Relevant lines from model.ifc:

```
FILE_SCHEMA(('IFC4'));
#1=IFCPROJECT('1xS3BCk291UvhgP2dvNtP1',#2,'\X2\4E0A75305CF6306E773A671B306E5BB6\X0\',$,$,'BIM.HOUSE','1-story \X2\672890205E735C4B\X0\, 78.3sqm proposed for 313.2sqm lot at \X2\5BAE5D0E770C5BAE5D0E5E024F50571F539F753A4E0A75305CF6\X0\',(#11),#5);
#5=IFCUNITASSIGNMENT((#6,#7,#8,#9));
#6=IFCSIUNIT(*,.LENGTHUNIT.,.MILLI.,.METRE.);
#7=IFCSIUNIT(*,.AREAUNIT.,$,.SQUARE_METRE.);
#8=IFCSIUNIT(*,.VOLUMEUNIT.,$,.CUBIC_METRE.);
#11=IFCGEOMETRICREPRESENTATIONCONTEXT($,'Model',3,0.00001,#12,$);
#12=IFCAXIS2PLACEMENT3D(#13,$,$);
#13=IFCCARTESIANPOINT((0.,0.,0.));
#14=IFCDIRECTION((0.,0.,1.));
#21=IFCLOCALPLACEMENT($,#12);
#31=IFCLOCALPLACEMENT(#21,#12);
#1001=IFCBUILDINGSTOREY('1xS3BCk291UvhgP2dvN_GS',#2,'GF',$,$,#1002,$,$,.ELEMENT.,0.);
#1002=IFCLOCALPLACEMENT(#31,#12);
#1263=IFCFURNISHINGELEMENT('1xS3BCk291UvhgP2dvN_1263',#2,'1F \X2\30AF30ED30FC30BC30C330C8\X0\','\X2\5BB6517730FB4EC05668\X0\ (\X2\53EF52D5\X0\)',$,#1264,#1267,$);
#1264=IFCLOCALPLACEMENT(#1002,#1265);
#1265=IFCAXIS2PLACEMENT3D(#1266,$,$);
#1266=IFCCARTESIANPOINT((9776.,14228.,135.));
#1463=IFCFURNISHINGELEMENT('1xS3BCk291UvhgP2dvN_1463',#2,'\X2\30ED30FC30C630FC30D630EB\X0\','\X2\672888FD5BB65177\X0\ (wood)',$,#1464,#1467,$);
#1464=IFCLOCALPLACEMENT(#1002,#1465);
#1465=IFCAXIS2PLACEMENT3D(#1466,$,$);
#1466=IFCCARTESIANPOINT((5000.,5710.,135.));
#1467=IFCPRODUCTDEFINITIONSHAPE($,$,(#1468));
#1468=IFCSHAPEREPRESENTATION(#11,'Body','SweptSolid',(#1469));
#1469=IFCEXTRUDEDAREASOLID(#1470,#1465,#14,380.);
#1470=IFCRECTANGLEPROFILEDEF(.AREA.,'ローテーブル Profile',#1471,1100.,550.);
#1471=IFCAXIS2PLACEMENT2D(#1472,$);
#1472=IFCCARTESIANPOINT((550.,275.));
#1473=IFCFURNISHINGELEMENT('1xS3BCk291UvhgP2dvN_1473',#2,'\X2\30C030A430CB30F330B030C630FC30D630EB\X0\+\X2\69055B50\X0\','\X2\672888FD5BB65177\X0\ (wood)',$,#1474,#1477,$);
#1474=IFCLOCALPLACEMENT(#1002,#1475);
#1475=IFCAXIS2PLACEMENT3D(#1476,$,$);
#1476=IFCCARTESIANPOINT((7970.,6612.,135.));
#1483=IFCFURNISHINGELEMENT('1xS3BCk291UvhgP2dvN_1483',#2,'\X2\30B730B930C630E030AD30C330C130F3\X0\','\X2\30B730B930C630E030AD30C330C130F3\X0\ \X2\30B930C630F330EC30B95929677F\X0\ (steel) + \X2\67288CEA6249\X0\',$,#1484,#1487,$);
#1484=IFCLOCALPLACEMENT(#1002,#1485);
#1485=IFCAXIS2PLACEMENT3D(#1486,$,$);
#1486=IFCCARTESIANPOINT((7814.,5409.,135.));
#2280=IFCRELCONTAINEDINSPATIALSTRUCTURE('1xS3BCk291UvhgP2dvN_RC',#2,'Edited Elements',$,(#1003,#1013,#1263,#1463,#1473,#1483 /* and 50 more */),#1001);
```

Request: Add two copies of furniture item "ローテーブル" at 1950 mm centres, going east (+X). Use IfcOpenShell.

```python
import numpy as np
import ifcopenshell
import ifcopenshell.api.geometry
import ifcopenshell.api.root
import ifcopenshell.util.element
import ifcopenshell.util.placement
import ifcopenshell.util.unit

model = ifcopenshell.open("model.ifc")
unit_scale = ifcopenshell.util.unit.calculate_unit_scale(model)


def reuse_history(source, copy):
    """copy_class also copies each property set's owner history, people and application; keep the originals."""
    for rel in copy.IsDefinedBy:
        if rel.is_a("IfcRelDefinesByProperties") and (history := rel.RelatingPropertyDefinition.OwnerHistory):
            rel.RelatingPropertyDefinition.OwnerHistory = source.OwnerHistory
            ifcopenshell.util.element.remove_deep2(model, history)


source = model.by_guid("1xS3BCk291UvhgP2dvN_1463")
base = ifcopenshell.util.placement.get_local_placement(source.ObjectPlacement)
step = np.array([1.0, 0.0, 0.0]) * 1.95 / unit_scale

for i in range(1, 3):
    copy = ifcopenshell.api.root.copy_class(model, product=source)
    copy.Representation = ifcopenshell.util.element.copy_deep(
        model, source.Representation, exclude=["IfcGeometricRepresentationContext", "IfcRepresentationMap"]
    )
    reuse_history(source, copy)
    matrix = base.copy()
    matrix[:3, 3] += i * step
    print("added at", matrix[:3, 3].round(3) + 0.0)
    ifcopenshell.api.geometry.edit_object_placement(model, product=copy, matrix=matrix, is_si=False)

model.write("model-out.ifc")
```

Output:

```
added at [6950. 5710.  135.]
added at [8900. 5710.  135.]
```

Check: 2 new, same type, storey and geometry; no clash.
